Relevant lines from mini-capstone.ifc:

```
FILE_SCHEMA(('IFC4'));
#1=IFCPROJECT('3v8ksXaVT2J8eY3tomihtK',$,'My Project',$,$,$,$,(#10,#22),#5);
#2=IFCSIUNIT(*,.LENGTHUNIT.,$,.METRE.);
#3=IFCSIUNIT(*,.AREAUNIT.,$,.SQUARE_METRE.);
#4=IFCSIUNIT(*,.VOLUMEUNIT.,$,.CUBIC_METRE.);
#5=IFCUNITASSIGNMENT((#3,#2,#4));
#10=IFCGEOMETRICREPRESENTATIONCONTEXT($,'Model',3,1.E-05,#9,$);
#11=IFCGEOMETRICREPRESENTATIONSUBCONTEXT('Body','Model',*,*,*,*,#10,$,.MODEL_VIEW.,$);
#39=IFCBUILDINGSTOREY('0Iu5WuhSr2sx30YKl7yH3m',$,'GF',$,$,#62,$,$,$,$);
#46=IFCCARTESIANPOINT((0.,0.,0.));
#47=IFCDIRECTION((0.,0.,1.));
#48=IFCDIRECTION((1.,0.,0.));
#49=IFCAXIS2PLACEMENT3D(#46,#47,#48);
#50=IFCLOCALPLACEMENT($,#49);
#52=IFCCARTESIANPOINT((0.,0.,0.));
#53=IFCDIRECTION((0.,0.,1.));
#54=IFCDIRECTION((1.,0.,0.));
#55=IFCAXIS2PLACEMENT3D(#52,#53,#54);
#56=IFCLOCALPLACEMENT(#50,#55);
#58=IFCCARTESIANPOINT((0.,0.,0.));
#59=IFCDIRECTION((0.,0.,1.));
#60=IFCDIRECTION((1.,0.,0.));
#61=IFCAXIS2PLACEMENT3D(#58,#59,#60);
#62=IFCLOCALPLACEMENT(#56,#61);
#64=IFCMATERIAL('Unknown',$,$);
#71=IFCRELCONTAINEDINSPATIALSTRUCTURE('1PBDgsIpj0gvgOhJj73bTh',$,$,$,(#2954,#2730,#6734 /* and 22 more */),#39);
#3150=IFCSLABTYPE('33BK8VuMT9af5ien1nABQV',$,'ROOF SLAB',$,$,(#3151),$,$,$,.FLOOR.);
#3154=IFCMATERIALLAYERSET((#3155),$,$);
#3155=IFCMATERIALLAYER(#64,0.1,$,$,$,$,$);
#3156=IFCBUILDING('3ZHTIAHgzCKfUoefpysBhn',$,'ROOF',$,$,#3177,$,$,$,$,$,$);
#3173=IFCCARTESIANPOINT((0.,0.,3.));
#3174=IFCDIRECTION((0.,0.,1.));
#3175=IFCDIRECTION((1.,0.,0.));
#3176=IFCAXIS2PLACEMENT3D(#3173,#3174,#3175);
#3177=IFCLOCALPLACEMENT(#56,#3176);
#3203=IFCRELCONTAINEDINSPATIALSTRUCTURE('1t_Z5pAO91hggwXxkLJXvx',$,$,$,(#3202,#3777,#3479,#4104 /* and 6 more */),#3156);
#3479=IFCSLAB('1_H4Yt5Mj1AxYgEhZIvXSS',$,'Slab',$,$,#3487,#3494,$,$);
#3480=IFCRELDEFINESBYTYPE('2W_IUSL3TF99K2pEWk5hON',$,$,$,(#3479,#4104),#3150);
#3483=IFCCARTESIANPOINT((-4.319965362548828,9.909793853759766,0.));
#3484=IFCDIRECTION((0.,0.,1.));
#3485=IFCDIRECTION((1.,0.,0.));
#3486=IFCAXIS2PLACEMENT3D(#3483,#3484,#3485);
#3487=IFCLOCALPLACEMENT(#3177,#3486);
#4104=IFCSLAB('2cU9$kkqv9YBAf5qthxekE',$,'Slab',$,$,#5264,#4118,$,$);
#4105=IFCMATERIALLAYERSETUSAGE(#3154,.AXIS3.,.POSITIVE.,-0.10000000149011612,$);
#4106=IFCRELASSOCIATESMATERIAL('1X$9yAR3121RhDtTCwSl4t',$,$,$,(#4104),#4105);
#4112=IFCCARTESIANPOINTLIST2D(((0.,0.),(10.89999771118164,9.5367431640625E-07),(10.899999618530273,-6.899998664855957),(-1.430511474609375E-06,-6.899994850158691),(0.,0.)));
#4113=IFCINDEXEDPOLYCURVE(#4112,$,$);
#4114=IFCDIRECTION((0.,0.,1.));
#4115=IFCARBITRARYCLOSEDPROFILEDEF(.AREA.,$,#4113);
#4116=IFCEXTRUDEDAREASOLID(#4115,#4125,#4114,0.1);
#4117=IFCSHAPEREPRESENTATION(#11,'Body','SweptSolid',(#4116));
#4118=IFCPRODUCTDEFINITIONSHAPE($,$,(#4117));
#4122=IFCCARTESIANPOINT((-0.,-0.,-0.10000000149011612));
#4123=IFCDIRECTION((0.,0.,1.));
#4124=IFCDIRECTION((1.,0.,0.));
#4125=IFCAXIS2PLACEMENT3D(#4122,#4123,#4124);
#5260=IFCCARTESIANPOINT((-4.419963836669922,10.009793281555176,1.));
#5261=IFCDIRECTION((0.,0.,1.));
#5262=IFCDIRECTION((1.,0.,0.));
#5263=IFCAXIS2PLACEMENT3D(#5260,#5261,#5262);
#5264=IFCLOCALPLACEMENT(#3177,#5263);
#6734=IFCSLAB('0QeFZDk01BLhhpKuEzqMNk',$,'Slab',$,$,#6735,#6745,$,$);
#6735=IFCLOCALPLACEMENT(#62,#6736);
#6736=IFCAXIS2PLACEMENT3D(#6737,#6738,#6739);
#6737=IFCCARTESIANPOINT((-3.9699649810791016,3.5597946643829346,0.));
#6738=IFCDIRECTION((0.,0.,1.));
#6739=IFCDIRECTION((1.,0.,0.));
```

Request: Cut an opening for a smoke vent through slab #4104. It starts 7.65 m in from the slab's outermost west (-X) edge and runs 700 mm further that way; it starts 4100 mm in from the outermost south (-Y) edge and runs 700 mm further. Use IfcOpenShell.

```python
import numpy as np
import ifcopenshell
import ifcopenshell.api.feature
import ifcopenshell.api.geometry
import ifcopenshell.api.root
import ifcopenshell.geom
import ifcopenshell.util.placement
import ifcopenshell.util.representation
import ifcopenshell.util.shape
import ifcopenshell.util.unit

model = ifcopenshell.open("mini-capstone.ifc")
unit_scale = ifcopenshell.util.unit.calculate_unit_scale(model)
settings = ifcopenshell.geom.settings()


def volume(element):
    """Net volume in cubic metres, openings subtracted."""
    shape = ifcopenshell.geom.create_shape(settings, element)
    return ifcopenshell.util.shape.get_volume(shape.geometry)


slab = model.by_guid("2cU9$kkqv9YBAf5qthxekE")
before = volume(slab)

# Extent in the slab's own axes, in metres. The edges named are its -X and -Y sides.
slab_shape = ifcopenshell.geom.create_shape(settings, slab)
vertices = ifcopenshell.util.shape.get_vertices(slab_shape.geometry)
x_min, y_min, bottom = vertices.min(axis=0)
top = vertices[:, 2].max()

opening = ifcopenshell.api.root.create_entity(model, ifc_class="IfcOpeningElement", name="Smoke vent opening", predefined_type="OPENING")
context = ifcopenshell.util.representation.get_context(model, "Model", "Body", "MODEL_VIEW")
width, depth = 0.7, 0.7
outline = [(0.0, 0.0), (width, 0.0), (width, depth), (0.0, depth), (0.0, 0.0)]
# Overshoot both faces by 50 mm so the cut is clean.
shape = ifcopenshell.api.geometry.add_slab_representation(
    model, context=context, depth=top - bottom + 0.1, polyline=outline
)
ifcopenshell.api.geometry.assign_representation(model, product=opening, representation=shape)

matrix = ifcopenshell.util.placement.get_local_placement(slab.ObjectPlacement)
matrix[:, 3] = matrix @ np.append(np.array([x_min + 7.65, y_min + 4.1, bottom - 0.05]) / unit_scale, 1.0)
ifcopenshell.api.geometry.edit_object_placement(model, product=opening, matrix=matrix, is_si=False)
ifcopenshell.api.feature.add_feature(model, feature=opening, element=slab)

after = volume(slab)

print(f"slab volume {before:.3f} -> {after:.3f} m3")

model.write("mini-capstone_updated.ifc")
```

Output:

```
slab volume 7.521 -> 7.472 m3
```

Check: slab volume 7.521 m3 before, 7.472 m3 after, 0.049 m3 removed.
